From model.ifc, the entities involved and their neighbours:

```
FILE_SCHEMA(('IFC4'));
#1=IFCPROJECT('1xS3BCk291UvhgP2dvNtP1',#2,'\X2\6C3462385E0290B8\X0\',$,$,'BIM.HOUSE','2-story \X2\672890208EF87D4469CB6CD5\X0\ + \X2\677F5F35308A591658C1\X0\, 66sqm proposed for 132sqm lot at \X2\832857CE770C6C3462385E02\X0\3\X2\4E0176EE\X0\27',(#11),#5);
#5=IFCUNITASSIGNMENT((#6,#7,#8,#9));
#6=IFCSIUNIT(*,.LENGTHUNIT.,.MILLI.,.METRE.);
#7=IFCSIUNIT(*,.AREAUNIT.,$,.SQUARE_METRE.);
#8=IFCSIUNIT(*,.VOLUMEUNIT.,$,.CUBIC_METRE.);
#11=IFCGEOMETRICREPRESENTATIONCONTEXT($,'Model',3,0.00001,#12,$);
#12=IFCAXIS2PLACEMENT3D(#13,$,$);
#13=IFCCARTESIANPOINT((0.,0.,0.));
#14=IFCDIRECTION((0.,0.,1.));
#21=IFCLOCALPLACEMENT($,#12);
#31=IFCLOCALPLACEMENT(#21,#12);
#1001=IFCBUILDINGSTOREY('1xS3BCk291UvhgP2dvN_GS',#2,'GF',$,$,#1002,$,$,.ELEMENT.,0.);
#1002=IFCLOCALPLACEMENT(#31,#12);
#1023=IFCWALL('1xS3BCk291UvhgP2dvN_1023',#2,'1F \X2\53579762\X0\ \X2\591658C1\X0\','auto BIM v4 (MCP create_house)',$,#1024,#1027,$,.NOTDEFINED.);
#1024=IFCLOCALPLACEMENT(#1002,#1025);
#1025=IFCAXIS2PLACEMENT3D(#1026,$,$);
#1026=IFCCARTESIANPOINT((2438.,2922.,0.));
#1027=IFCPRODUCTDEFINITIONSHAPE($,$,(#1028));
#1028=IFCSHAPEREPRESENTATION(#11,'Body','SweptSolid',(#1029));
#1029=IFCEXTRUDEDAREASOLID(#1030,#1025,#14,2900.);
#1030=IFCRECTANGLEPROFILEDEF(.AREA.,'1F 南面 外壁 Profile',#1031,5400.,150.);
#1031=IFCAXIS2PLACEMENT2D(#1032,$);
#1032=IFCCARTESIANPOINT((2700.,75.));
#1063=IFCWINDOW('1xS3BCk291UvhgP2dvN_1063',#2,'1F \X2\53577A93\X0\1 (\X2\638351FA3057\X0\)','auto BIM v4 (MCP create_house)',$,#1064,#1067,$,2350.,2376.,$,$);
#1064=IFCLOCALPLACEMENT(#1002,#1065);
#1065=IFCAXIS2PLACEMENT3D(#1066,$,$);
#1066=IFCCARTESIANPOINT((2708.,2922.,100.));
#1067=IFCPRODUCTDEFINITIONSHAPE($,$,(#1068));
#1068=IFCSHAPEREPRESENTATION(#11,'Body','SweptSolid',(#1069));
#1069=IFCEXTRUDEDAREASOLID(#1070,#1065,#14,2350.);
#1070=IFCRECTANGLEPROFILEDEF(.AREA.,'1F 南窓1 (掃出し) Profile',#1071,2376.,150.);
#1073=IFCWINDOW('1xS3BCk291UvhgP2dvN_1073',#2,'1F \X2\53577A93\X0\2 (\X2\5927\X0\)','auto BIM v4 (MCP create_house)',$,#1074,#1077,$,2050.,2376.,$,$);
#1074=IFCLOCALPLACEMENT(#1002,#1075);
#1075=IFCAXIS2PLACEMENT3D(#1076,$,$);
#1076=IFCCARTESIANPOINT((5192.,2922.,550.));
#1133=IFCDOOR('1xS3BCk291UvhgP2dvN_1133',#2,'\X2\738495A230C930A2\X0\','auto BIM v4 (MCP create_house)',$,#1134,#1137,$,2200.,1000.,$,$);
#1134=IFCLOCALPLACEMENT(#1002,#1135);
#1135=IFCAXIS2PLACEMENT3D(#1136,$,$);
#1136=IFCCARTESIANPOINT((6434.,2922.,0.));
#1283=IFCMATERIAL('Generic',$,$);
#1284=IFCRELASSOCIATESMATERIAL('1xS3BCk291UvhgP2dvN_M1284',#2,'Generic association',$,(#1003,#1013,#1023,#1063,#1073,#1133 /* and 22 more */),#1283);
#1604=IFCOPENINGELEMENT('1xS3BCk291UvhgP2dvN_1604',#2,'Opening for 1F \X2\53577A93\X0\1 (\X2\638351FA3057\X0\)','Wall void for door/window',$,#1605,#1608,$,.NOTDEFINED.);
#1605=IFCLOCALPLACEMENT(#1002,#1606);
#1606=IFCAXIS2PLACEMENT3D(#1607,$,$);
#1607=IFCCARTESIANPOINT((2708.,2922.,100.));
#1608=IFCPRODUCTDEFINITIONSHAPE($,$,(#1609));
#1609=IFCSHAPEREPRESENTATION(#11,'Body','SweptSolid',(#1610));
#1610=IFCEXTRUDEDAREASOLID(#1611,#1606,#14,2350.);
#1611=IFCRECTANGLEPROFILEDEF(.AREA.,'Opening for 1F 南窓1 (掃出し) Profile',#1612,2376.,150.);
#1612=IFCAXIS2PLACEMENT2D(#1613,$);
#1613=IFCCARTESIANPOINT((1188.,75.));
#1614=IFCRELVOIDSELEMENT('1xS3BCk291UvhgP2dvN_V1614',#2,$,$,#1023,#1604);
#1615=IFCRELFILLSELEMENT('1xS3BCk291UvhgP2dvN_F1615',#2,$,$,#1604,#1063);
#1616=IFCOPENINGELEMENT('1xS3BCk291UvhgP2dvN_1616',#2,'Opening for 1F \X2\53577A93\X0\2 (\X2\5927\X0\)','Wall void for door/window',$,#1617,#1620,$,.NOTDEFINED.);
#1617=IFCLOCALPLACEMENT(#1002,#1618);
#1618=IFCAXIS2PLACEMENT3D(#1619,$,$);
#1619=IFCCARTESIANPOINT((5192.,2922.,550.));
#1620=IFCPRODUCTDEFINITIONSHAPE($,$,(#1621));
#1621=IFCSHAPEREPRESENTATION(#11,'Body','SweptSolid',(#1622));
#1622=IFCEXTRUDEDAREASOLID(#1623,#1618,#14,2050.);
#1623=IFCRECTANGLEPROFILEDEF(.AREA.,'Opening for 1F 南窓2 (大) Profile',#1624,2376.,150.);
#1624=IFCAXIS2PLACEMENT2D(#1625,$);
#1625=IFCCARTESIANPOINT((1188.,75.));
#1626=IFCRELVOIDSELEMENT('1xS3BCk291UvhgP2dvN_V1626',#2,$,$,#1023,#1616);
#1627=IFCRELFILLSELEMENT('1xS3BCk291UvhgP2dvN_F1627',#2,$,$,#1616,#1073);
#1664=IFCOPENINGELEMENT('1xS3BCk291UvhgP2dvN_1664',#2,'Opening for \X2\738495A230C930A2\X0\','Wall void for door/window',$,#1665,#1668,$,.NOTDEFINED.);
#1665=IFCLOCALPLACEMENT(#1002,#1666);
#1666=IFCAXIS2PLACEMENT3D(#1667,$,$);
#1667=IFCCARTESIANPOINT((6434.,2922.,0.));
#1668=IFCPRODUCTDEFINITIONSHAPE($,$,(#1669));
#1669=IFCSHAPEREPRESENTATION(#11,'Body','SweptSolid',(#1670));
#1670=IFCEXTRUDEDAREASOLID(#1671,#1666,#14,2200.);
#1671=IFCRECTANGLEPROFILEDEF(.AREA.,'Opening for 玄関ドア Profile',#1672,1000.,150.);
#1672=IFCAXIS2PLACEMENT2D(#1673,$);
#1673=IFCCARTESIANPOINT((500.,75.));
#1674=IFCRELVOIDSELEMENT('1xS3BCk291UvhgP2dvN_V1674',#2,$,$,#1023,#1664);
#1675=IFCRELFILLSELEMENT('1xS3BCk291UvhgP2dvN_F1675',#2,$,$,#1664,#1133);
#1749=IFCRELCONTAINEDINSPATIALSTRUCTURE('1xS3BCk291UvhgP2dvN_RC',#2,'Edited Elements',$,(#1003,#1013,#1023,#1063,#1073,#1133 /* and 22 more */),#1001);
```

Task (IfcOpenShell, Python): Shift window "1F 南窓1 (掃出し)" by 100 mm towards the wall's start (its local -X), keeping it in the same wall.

```python
import ifcopenshell
import ifcopenshell.api.geometry
import ifcopenshell.util.placement

model = ifcopenshell.open("model.ifc")

window = model.by_guid("1xS3BCk291UvhgP2dvN_1063")
opening = window.FillsVoids[0].RelatingOpeningElement
wall = opening.VoidsElements[0].RelatingBuildingElement

wall_matrix = ifcopenshell.util.placement.get_local_placement(wall.ObjectPlacement)
shift = wall_matrix[:3, 0] * -100.0
before = ifcopenshell.util.placement.get_local_placement(window.ObjectPlacement)[:3, 3].copy()

# The window is not placed relative to its opening, so move both.
for product in (opening, window):
    matrix = ifcopenshell.util.placement.get_local_placement(product.ObjectPlacement)
    matrix[:3, 3] += shift
    ifcopenshell.api.geometry.edit_object_placement(model, product=product, matrix=matrix, is_si=False)

after = ifcopenshell.util.placement.get_local_placement(window.ObjectPlacement)[:3, 3]
print("window moved by", (after - before).round(3) + 0.0)

model.write("model-out.ifc")
```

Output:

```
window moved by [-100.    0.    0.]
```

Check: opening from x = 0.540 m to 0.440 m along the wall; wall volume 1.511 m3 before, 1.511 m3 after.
